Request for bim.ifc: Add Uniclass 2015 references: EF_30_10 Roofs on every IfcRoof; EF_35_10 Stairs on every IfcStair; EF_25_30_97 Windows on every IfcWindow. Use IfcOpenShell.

First a look at what the model holds.

```python
import ifcopenshell

model = ifcopenshell.open("bim.ifc")
print(model.schema)
print("classifications:", [c.Name for c in model.by_type("IfcClassification")])
for ifc_class in ("IfcDoor", "IfcRoof", "IfcStair", "IfcWall", "IfcWindow"):
    print(ifc_class, len(model.by_type(ifc_class)))
```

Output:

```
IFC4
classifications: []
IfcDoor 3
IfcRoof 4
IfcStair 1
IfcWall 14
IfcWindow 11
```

```python
import ifcopenshell
import ifcopenshell.api.classification

model = ifcopenshell.open("bim.ifc")

system = ifcopenshell.api.classification.add_classification(model, classification="Uniclass 2015")

codes = {
    "IfcRoof": ("EF_30_10", "Roofs"),
    "IfcStair": ("EF_35_10", "Stairs"),
    "IfcWindow": ("EF_25_30_97", "Windows"),
}
for ifc_class, (code, name) in codes.items():
    products = model.by_type(ifc_class)
    ifcopenshell.api.classification.add_reference(
        model, products=products, classification=system, identification=code, name=name
    )
    print(code, len(products))

model.write("bim_v2.ifc")
```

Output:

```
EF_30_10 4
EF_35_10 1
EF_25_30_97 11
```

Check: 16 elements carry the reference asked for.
